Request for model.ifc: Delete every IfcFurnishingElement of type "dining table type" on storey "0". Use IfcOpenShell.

First a look at what the model holds.

```python
import ifcopenshell
import ifcopenshell.util.element

model = ifcopenshell.open("model.ifc")
print(model.schema)
storey = next(s for s in model.by_type("IfcBuildingStorey") if s.Name == "0")
furniture = [e for e in ifcopenshell.util.element.get_decomposition(storey) if e.is_a("IfcFurnishingElement")]
seen = {}
for e in furniture:
    element_type = ifcopenshell.util.element.get_type(e)
    name = element_type.Name if element_type not in (None, e) else None
    seen[name] = seen.get(name, 0) + 1
for name, count in sorted(seen.items(), key=str):
    print(count, "x", name)
```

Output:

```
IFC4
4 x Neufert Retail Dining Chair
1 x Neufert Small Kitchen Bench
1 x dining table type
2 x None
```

```python
import ifcopenshell
import ifcopenshell.api.root
import ifcopenshell.util.element

model = ifcopenshell.open("model.ifc")

storey = next(s for s in model.by_type("IfcBuildingStorey") if s.Name == "0")
furniture = [e for e in ifcopenshell.util.element.get_decomposition(storey) if e.is_a("IfcFurnishingElement")]
targets = [e for e in furniture if (t := ifcopenshell.util.element.get_type(e)) not in (None, e) and t.Name == "dining table type"]

for e in targets:
    ifcopenshell.api.root.remove_product(model, product=e)
print(len(targets), "removed")

model.write("model_rev.ifc")
```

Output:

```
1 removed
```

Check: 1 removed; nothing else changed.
